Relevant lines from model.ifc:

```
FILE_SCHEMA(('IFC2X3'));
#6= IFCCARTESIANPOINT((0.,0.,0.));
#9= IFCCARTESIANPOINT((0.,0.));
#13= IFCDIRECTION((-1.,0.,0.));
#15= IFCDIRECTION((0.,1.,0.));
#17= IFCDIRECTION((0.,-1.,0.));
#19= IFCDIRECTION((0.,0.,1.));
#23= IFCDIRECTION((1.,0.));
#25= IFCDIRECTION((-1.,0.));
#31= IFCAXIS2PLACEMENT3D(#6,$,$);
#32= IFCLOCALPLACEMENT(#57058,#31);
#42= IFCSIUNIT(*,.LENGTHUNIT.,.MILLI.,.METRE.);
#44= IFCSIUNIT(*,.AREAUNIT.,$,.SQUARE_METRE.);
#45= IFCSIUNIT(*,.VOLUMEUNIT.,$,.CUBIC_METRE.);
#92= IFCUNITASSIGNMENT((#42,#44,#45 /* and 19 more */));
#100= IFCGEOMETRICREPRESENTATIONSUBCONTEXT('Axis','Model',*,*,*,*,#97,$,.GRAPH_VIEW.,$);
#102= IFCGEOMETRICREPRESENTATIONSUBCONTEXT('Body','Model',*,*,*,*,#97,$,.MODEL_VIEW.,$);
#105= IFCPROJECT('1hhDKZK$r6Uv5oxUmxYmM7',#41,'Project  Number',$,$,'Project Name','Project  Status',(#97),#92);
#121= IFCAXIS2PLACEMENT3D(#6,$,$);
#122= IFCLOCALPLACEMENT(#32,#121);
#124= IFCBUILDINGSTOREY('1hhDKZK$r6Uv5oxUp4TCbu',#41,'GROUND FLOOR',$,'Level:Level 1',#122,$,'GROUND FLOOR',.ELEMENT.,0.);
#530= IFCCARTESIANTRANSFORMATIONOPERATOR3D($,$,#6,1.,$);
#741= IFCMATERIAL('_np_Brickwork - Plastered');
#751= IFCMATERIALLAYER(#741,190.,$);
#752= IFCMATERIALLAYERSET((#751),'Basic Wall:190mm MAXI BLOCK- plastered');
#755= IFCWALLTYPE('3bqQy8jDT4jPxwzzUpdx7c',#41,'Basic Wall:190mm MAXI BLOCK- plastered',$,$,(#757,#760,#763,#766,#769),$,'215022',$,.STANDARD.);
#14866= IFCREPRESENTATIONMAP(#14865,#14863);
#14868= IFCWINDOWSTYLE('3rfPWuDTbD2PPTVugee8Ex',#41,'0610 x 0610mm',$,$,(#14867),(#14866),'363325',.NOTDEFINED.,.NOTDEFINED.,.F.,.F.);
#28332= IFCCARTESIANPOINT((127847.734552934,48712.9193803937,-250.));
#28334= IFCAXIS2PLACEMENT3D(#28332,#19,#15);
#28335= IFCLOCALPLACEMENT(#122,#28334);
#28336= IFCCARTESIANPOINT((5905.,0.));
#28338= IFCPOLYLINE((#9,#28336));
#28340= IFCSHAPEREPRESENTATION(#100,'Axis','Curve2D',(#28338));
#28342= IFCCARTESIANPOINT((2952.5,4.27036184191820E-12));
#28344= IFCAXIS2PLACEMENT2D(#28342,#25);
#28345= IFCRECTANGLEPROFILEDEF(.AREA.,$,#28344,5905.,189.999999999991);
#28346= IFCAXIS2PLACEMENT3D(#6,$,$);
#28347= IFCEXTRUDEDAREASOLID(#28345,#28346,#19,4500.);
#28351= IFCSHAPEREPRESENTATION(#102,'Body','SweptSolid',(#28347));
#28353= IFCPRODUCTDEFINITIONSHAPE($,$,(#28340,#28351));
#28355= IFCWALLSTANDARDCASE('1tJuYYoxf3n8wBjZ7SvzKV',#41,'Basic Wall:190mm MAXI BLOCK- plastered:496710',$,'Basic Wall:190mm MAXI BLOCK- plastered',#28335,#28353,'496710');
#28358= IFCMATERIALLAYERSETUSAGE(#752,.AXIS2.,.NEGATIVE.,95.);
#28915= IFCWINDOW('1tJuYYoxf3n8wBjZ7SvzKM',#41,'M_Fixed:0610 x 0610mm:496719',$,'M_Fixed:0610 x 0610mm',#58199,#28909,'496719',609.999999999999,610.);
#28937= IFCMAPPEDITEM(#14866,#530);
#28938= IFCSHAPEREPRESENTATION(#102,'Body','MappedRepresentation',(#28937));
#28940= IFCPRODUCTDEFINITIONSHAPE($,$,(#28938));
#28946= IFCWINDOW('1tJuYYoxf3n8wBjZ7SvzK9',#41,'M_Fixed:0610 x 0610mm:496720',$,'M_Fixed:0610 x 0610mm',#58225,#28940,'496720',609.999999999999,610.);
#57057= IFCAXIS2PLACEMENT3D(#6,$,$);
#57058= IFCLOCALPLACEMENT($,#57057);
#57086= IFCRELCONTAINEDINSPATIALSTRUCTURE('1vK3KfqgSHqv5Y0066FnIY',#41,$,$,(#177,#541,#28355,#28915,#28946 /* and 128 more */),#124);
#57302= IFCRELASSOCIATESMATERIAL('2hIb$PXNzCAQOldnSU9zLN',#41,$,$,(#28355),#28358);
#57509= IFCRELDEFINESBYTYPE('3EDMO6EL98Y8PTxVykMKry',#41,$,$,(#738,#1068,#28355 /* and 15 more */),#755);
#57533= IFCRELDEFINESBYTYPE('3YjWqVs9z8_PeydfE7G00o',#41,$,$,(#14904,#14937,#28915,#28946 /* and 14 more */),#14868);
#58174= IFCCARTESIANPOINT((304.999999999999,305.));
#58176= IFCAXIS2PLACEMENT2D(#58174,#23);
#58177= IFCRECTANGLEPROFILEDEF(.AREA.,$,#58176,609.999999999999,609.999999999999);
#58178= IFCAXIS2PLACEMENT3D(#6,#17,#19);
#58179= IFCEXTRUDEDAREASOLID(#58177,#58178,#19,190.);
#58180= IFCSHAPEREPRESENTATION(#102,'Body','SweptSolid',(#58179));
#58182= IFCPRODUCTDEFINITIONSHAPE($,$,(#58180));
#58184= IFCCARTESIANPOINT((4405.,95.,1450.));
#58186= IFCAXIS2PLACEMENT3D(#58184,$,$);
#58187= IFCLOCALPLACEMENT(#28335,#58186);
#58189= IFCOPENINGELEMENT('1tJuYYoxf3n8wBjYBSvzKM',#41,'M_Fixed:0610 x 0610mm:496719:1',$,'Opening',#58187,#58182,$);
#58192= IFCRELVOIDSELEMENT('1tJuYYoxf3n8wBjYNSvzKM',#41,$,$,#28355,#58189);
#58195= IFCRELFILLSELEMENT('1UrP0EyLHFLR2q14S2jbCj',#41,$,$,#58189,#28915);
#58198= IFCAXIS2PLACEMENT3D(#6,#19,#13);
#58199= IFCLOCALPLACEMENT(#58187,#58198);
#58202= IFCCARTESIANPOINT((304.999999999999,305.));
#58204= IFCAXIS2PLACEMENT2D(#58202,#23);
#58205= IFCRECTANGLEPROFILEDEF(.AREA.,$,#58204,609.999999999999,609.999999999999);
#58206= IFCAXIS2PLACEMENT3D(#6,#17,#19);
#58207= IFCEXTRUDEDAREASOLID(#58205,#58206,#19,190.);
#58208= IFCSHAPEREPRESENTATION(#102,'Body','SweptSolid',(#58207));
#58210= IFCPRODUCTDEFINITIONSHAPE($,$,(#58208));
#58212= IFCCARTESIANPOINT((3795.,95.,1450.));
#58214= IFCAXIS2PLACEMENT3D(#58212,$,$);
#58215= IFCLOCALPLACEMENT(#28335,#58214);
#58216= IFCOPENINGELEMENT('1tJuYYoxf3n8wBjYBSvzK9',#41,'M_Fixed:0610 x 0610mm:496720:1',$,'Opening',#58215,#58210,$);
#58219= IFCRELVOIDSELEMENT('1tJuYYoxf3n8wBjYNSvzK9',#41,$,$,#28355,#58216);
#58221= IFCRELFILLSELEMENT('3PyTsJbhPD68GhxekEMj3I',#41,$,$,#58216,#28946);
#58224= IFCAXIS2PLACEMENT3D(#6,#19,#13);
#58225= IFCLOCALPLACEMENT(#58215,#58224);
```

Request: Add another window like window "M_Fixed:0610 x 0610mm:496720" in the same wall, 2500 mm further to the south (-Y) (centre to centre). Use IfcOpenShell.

```python
import ifcopenshell
import ifcopenshell.api.feature
import ifcopenshell.api.geometry
import ifcopenshell.api.root
import ifcopenshell.geom
import ifcopenshell.util.element
import ifcopenshell.util.placement
import ifcopenshell.util.shape
import ifcopenshell.util.unit

model = ifcopenshell.open("model.ifc")
unit_scale = ifcopenshell.util.unit.calculate_unit_scale(model)
settings = ifcopenshell.geom.settings()


def volume(element):
    """Net volume in cubic metres, openings subtracted."""
    shape = ifcopenshell.geom.create_shape(settings, element)
    return ifcopenshell.util.shape.get_volume(shape.geometry)


def reuse_history(source, copy):
    """copy_class also copies each property set's owner history, people and application; keep the originals."""
    for rel in copy.IsDefinedBy:
        if rel.is_a("IfcRelDefinesByProperties") and (history := rel.RelatingPropertyDefinition.OwnerHistory):
            rel.RelatingPropertyDefinition.OwnerHistory = source.OwnerHistory
            ifcopenshell.util.element.remove_deep2(model, history)


window = model.by_guid("1tJuYYoxf3n8wBjZ7SvzK9")
opening = window.FillsVoids[0].RelatingOpeningElement
wall = opening.VoidsElements[0].RelatingBuildingElement
before = volume(wall)
shift = ifcopenshell.util.placement.get_local_placement(wall.ObjectPlacement)[:3, 0] * -2.5 / unit_scale

# copy_class copies the void relationship, type, container and properties, but no geometry.
new_opening = ifcopenshell.api.root.copy_class(model, product=opening)
new_opening.Representation = ifcopenshell.util.element.copy_deep(
    model, opening.Representation, exclude=["IfcGeometricRepresentationContext", "IfcRepresentationMap"]
)
new_opening.Name = "M_Fixed:0610 x 0610mm"
new_window = ifcopenshell.api.root.copy_class(model, product=window)
new_window.Representation = ifcopenshell.util.element.copy_deep(
    model, window.Representation, exclude=["IfcGeometricRepresentationContext", "IfcRepresentationMap"]
)
new_window.Name = "M_Fixed:0610 x 0610mm"
new_window.Tag = None
reuse_history(window, new_window)
fills = ifcopenshell.api.feature.add_filling(model, opening=new_opening, element=new_window)
fills.OwnerHistory = new_window.OwnerHistory  # required in IFC2X3

for old, new in ((opening, new_opening), (window, new_window)):
    matrix = ifcopenshell.util.placement.get_local_placement(old.ObjectPlacement)
    matrix[:3, 3] += shift
    ifcopenshell.api.geometry.edit_object_placement(model, product=new, matrix=matrix, is_si=False)

after = volume(wall)

print(f"wall volume {before:.3f} -> {after:.3f} m3")

model.write("model_rev.ifc")
```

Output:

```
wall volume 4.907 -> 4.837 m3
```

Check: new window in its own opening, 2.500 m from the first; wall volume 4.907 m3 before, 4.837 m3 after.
